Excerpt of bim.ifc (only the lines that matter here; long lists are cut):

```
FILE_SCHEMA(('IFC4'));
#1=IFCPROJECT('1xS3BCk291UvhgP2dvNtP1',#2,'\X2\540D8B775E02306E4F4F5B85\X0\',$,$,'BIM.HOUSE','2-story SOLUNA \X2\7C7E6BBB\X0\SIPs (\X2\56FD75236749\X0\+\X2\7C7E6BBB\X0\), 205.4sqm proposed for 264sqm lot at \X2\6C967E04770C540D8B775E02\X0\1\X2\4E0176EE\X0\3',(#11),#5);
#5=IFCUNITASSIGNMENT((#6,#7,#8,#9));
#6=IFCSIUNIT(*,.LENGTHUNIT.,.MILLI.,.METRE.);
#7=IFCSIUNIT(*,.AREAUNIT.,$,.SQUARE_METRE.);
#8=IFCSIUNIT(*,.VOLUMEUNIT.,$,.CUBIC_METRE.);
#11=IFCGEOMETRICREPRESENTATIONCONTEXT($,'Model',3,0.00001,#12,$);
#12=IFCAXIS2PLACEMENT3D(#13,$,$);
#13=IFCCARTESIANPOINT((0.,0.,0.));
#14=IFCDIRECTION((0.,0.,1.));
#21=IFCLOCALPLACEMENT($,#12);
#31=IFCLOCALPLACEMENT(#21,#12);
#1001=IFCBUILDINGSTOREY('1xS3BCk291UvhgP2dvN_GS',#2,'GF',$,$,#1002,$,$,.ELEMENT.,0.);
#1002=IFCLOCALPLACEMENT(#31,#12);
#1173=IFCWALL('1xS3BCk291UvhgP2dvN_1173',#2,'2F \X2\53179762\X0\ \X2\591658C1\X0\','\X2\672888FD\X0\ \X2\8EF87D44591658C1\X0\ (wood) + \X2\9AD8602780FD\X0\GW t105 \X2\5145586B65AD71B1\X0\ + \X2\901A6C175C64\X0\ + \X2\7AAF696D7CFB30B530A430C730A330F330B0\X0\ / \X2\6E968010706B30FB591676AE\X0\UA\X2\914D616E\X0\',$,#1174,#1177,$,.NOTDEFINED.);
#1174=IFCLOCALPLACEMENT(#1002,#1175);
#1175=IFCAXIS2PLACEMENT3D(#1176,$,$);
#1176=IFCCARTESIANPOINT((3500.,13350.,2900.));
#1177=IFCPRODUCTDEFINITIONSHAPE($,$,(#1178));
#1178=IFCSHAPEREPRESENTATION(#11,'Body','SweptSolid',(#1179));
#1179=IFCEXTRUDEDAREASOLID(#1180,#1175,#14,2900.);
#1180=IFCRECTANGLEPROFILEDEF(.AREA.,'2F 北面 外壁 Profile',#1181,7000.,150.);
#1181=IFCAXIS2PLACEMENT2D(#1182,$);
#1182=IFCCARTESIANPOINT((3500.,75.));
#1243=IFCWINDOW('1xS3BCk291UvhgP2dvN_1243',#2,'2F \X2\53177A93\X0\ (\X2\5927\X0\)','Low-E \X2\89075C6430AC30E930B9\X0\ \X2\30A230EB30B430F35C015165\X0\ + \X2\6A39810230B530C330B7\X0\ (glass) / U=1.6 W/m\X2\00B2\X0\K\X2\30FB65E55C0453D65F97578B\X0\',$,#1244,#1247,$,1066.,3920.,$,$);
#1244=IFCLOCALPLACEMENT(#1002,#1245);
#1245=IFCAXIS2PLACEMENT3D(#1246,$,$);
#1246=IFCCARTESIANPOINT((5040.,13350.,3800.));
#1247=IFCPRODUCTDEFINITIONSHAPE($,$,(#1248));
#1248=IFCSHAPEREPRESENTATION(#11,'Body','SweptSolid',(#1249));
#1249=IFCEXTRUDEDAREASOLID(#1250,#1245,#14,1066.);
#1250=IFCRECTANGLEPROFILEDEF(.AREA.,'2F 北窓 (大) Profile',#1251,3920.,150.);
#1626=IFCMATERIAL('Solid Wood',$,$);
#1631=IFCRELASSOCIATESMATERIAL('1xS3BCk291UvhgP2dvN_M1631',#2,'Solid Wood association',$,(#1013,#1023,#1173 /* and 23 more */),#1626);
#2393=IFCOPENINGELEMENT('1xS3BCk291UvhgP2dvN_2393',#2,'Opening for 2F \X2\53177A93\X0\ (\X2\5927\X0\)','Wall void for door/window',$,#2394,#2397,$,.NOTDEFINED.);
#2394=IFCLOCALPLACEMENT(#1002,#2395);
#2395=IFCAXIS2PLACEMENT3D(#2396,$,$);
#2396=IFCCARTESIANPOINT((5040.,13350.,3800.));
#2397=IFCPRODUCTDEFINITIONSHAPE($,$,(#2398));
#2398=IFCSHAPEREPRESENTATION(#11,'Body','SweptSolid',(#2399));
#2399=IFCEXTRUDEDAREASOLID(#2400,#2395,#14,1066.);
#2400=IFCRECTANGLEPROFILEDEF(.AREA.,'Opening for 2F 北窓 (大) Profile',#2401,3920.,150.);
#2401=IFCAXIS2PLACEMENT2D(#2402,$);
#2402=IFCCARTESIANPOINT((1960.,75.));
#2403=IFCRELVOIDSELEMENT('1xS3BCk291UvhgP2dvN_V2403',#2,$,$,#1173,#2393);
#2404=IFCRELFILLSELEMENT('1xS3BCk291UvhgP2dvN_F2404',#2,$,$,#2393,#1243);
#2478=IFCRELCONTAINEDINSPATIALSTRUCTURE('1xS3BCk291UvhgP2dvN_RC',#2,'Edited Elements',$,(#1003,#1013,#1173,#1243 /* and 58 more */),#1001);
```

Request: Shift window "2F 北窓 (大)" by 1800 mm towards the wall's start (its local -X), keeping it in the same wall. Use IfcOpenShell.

```python
import ifcopenshell
import ifcopenshell.api.geometry
import ifcopenshell.util.placement
import ifcopenshell.util.unit

model = ifcopenshell.open("bim.ifc")
unit_scale = ifcopenshell.util.unit.calculate_unit_scale(model)

window = model.by_guid("1xS3BCk291UvhgP2dvN_1243")
opening = window.FillsVoids[0].RelatingOpeningElement
wall = opening.VoidsElements[0].RelatingBuildingElement

wall_matrix = ifcopenshell.util.placement.get_local_placement(wall.ObjectPlacement)
shift = wall_matrix[:3, 0] * -1.8 / unit_scale
before = ifcopenshell.util.placement.get_local_placement(window.ObjectPlacement)[:3, 3].copy()

# The window is not placed relative to its opening, so move both.
for product in (opening, window):
    matrix = ifcopenshell.util.placement.get_local_placement(product.ObjectPlacement)
    matrix[:3, 3] += shift
    ifcopenshell.api.geometry.edit_object_placement(model, product=product, matrix=matrix, is_si=False)

after = ifcopenshell.util.placement.get_local_placement(window.ObjectPlacement)[:3, 3]
print("window moved by", (after - before).round(3) + 0.0)

model.write("bim-out.ifc")
```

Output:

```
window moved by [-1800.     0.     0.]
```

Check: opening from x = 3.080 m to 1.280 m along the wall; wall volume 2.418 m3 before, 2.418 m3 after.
